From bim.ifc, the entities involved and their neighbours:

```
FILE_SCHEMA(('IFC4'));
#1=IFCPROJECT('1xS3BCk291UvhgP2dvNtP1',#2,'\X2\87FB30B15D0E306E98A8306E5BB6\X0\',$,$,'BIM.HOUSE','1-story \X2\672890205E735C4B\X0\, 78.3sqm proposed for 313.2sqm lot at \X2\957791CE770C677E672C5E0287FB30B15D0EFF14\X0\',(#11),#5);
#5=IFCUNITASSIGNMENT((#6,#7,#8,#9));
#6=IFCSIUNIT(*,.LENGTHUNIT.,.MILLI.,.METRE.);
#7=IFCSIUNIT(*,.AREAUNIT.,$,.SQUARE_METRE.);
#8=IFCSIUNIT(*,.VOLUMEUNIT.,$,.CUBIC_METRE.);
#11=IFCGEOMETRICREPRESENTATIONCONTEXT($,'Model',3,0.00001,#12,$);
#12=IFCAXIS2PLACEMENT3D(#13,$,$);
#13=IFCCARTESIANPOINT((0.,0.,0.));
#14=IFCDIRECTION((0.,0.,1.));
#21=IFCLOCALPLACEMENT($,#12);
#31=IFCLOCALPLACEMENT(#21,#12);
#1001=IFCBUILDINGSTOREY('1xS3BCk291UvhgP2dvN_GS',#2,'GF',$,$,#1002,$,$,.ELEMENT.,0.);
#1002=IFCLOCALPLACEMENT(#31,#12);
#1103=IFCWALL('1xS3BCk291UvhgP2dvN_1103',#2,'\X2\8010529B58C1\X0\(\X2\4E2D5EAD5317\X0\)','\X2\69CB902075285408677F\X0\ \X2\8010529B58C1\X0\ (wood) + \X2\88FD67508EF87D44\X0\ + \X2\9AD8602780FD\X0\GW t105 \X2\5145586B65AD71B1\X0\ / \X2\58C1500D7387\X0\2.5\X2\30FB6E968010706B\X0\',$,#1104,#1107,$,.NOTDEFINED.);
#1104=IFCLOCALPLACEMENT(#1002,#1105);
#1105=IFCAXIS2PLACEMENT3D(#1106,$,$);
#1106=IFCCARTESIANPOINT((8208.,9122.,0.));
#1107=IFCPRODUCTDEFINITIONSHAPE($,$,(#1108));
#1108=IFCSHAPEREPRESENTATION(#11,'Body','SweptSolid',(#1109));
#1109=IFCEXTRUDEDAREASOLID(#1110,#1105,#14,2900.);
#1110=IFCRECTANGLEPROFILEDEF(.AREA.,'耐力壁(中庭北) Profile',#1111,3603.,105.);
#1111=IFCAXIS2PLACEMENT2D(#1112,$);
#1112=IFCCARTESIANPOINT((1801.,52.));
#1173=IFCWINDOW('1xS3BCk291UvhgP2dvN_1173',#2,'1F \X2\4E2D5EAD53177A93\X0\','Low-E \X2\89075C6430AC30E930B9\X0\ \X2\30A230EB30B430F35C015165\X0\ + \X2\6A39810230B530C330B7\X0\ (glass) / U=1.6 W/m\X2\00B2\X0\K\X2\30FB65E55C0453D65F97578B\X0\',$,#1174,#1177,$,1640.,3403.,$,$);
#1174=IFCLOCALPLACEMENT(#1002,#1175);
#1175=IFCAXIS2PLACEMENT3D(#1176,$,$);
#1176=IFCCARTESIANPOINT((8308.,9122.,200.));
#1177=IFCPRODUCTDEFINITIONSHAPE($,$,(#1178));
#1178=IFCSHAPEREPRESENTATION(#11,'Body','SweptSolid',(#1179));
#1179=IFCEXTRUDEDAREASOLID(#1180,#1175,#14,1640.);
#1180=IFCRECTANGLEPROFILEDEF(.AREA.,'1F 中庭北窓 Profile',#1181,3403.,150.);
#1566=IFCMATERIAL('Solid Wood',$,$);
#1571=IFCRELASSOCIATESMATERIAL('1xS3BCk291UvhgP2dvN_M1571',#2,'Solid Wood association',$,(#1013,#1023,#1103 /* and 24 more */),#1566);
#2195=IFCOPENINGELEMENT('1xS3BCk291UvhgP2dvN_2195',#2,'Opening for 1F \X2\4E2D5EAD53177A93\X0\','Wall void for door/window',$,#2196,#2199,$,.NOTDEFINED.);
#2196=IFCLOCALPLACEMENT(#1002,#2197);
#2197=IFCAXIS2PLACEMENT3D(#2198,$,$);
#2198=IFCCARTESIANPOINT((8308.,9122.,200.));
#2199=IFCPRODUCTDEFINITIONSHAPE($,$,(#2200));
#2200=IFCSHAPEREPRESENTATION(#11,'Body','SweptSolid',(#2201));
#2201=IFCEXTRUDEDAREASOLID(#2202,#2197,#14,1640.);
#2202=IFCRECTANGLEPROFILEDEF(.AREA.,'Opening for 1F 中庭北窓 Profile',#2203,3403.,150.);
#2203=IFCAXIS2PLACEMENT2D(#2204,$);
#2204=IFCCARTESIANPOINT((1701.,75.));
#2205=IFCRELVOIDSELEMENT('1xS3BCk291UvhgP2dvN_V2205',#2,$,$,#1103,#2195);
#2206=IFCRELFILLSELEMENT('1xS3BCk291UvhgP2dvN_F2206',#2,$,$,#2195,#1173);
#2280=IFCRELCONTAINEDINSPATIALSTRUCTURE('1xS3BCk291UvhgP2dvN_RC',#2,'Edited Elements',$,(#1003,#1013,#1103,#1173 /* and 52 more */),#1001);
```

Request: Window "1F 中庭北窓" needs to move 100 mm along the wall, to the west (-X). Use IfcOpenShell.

```python
import ifcopenshell
import ifcopenshell.api.geometry
import ifcopenshell.util.placement

model = ifcopenshell.open("bim.ifc")

window = model.by_guid("1xS3BCk291UvhgP2dvN_1173")
opening = window.FillsVoids[0].RelatingOpeningElement
wall = opening.VoidsElements[0].RelatingBuildingElement

wall_matrix = ifcopenshell.util.placement.get_local_placement(wall.ObjectPlacement)
shift = wall_matrix[:3, 0] * -100.0
before = ifcopenshell.util.placement.get_local_placement(window.ObjectPlacement)[:3, 3].copy()

# The window is not placed relative to its opening, so move both.
for product in (opening, window):
    matrix = ifcopenshell.util.placement.get_local_placement(product.ObjectPlacement)
    matrix[:3, 3] += shift
    ifcopenshell.api.geometry.edit_object_placement(model, product=product, matrix=matrix, is_si=False)

after = ifcopenshell.util.placement.get_local_placement(window.ObjectPlacement)[:3, 3]
print("window moved by", (after - before).round(3) + 0.0)

model.write("bim_updated.ifc")
```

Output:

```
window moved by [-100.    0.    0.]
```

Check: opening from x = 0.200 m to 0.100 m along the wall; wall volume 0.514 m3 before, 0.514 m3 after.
